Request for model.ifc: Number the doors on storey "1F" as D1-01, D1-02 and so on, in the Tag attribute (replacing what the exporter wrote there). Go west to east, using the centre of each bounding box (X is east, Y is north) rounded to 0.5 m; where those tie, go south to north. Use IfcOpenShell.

First a look at what the model holds.

```python
import ifcopenshell
import ifcopenshell.util.element
import ifcopenshell.util.placement

model = ifcopenshell.open("model.ifc")
print(model.schema)
storey = next(s for s in model.by_type("IfcBuildingStorey") if s.Name == "1F")
doors = [e for e in ifcopenshell.util.element.get_decomposition(storey) if e.is_a("IfcDoor")]
for e in sorted(doors, key=lambda e: e.id()):
    origin = ifcopenshell.util.placement.get_local_placement(e.ObjectPlacement)[:3, 3]
    print(e.id(), e.Tag, e.Name, origin.round(2) + 0.0, sep=" | ")
```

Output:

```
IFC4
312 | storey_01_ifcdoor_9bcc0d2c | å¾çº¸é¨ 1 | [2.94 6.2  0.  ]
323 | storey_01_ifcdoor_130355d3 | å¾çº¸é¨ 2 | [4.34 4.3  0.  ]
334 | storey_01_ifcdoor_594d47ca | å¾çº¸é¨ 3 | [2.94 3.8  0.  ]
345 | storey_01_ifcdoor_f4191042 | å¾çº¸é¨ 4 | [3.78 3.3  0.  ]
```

```python
import ifcopenshell
import ifcopenshell.geom
import ifcopenshell.util.element
import ifcopenshell.util.shape

model = ifcopenshell.open("model.ifc")
settings = ifcopenshell.geom.settings()
settings.set("use-world-coords", True)


def centre(element):
    shape = ifcopenshell.geom.create_shape(settings, element)
    return ifcopenshell.util.shape.get_bbox_centroid(shape.geometry)


storey = next(s for s in model.by_type("IfcBuildingStorey") if s.Name == "1F")
doors = [e for e in ifcopenshell.util.element.get_decomposition(storey) if e.is_a("IfcDoor")]

# Insertion points can sit at a corner or the storey origin, so sort by the geometry (in metres).
centres = {e: centre(e) for e in doors}
doors.sort(key=lambda e: (round(centres[e][0] / 0.5), centres[e][1]))

for i, e in enumerate(doors, start=1):
    number = f"D1-{i:02d}"
    e.Tag = number
    print(e.id(), number)

model.write("model-out.ifc")
```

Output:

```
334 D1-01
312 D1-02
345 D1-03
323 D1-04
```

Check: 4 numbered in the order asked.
